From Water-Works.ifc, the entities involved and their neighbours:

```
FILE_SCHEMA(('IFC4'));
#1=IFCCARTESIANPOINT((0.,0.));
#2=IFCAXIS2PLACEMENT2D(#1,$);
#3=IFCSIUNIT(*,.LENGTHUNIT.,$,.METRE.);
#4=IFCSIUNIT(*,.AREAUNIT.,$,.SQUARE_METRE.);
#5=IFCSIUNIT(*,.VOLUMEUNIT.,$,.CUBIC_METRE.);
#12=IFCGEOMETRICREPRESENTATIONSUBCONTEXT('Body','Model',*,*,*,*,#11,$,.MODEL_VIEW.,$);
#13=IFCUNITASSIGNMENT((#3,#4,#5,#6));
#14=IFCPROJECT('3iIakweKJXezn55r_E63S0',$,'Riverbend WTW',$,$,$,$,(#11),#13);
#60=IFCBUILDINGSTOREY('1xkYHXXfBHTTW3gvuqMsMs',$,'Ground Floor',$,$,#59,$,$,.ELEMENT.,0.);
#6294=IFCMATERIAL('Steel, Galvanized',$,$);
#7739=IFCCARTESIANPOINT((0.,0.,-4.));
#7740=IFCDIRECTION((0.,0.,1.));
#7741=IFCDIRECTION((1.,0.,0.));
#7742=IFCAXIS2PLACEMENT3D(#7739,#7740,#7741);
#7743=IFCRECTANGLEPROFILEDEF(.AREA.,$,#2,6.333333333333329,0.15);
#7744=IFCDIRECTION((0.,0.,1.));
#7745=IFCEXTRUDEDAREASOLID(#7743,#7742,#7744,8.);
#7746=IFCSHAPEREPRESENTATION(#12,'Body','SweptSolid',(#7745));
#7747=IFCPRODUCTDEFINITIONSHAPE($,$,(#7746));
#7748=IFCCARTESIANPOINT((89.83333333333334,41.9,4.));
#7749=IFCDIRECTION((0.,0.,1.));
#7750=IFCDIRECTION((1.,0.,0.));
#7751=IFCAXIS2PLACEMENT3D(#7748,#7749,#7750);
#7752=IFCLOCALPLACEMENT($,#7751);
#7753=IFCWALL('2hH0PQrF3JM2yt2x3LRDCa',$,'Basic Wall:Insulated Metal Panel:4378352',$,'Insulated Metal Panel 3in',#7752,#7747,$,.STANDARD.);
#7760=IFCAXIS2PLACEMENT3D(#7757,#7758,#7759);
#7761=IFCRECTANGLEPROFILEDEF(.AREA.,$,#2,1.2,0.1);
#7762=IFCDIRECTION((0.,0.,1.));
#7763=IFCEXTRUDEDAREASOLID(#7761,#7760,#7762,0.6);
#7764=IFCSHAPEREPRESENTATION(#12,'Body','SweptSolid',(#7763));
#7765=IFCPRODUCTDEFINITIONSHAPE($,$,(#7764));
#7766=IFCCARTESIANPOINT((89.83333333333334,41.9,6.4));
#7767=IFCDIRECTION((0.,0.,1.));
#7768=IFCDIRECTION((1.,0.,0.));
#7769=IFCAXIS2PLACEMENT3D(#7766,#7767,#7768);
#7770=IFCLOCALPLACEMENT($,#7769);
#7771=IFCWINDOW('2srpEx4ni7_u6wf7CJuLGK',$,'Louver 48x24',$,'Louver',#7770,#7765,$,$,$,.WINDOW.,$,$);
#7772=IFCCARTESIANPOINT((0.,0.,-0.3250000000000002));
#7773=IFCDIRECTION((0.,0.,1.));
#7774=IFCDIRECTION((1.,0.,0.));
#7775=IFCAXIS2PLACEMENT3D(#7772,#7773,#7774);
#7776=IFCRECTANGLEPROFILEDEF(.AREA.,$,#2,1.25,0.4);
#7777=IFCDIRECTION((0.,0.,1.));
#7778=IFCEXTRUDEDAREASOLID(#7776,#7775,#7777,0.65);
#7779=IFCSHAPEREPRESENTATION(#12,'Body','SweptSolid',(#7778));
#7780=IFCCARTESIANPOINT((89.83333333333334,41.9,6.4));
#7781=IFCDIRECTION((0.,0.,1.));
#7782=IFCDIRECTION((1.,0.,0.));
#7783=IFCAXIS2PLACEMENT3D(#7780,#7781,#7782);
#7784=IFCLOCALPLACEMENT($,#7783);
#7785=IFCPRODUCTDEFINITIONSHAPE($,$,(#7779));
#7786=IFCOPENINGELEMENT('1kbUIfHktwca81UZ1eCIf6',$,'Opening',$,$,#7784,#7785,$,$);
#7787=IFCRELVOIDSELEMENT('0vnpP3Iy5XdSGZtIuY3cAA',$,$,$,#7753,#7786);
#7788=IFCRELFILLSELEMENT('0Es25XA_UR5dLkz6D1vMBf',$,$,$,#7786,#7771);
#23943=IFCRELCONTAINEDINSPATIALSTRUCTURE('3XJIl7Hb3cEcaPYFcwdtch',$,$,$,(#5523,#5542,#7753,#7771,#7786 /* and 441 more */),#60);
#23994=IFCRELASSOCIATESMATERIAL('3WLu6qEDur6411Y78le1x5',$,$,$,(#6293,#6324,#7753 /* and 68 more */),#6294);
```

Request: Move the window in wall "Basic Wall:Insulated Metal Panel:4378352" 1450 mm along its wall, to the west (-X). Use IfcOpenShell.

```python
import ifcopenshell
import ifcopenshell.api.geometry
import ifcopenshell.util.placement

model = ifcopenshell.open("Water-Works.ifc")

window = model.by_guid("2srpEx4ni7_u6wf7CJuLGK")
opening = window.FillsVoids[0].RelatingOpeningElement
wall = opening.VoidsElements[0].RelatingBuildingElement

wall_matrix = ifcopenshell.util.placement.get_local_placement(wall.ObjectPlacement)
shift = wall_matrix[:3, 0] * -1.45
before = ifcopenshell.util.placement.get_local_placement(window.ObjectPlacement)[:3, 3].copy()

# The window is not placed relative to its opening, so move both.
for product in (opening, window):
    matrix = ifcopenshell.util.placement.get_local_placement(product.ObjectPlacement)
    matrix[:3, 3] += shift
    ifcopenshell.api.geometry.edit_object_placement(model, product=product, matrix=matrix, is_si=False)

after = ifcopenshell.util.placement.get_local_placement(window.ObjectPlacement)[:3, 3]
print("window moved by", (after - before).round(3) + 0.0)

model.write("Water-Works_updated.ifc")
```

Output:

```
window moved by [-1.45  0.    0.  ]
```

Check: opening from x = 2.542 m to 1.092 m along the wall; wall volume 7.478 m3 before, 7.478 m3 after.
